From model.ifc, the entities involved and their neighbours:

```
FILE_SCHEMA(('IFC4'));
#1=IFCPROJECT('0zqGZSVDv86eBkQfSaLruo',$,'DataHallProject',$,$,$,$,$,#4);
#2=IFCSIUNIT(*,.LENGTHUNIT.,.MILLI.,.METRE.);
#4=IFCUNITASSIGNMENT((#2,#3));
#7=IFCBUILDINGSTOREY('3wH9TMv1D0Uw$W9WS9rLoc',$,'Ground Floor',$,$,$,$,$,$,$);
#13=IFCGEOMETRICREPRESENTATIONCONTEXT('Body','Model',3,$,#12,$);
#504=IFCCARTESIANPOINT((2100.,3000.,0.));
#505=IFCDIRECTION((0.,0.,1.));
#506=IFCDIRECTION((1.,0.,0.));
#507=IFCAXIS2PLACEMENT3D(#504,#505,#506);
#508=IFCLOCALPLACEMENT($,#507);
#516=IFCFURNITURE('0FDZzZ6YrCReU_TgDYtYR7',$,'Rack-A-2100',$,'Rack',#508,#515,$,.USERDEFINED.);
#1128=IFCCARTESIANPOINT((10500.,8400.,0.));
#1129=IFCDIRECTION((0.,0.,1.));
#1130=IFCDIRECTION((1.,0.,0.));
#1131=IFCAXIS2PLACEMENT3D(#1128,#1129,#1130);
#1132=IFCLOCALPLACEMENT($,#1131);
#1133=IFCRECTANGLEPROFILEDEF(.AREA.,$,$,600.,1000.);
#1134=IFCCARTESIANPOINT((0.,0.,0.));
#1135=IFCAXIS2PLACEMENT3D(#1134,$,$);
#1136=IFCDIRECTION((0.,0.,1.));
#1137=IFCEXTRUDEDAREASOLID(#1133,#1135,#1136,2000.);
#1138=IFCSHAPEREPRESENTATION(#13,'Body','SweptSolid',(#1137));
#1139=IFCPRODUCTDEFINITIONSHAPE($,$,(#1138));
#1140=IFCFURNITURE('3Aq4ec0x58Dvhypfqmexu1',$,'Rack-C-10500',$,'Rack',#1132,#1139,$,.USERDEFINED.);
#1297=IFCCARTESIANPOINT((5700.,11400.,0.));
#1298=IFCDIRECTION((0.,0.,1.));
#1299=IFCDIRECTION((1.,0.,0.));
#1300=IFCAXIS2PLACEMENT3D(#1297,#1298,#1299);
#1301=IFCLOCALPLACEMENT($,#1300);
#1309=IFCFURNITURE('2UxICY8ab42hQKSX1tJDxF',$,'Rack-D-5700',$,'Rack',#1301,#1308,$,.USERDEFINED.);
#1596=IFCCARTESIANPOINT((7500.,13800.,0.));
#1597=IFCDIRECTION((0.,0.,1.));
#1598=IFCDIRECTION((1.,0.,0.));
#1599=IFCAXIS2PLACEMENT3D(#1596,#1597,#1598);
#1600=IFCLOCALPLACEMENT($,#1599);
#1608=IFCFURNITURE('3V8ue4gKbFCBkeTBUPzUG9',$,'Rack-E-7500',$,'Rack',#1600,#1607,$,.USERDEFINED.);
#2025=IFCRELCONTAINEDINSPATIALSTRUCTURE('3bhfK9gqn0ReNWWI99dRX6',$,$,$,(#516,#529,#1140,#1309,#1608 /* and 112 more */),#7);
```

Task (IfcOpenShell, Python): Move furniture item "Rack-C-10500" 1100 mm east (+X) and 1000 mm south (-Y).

```python
import ifcopenshell
import ifcopenshell.api.geometry
import ifcopenshell.util.placement
import ifcopenshell.util.unit

model = ifcopenshell.open("model.ifc")
unit_scale = ifcopenshell.util.unit.calculate_unit_scale(model)

item = model.by_guid("3Aq4ec0x58Dvhypfqmexu1")
matrix = ifcopenshell.util.placement.get_local_placement(item.ObjectPlacement)
matrix[0, 3] += 1.1 / unit_scale
matrix[1, 3] -= 1 / unit_scale
ifcopenshell.api.geometry.edit_object_placement(model, product=item, matrix=matrix, is_si=False)

print(ifcopenshell.util.placement.get_local_placement(item.ObjectPlacement).round(3) + 0.0)

model.write("model_updated.ifc")
```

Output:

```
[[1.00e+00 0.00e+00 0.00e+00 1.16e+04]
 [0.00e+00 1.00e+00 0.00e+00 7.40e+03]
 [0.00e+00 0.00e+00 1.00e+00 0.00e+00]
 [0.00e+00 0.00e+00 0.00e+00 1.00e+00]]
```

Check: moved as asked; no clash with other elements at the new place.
